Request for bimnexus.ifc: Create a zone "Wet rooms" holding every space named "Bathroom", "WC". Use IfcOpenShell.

First a look at what the model holds.

```python
import ifcopenshell

model = ifcopenshell.open("bimnexus.ifc")
print(model.schema)
seen = {}
for space in model.by_type("IfcSpace"):
    seen[space.LongName] = seen.get(space.LongName, 0) + 1
for name, count in sorted(seen.items(), key=str):
    print(count, "x", name)
print("zones:", [z.Name for z in model.by_type("IfcZone")][:20])
```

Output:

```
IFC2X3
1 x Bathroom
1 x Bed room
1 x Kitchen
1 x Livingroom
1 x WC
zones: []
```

```python
import ifcopenshell
import ifcopenshell.api.group
import ifcopenshell.api.root

model = ifcopenshell.open("bimnexus.ifc")

names = {"Bathroom", "WC"}
spaces = [s for s in model.by_type("IfcSpace") if s.LongName in names]

zone = ifcopenshell.api.root.create_entity(model, ifc_class="IfcZone", name="Wet rooms")
ifcopenshell.api.group.assign_group(model, products=spaces, group=zone)
print(len(spaces), "spaces in", zone.Name)

model.write("bimnexus_rev.ifc")
```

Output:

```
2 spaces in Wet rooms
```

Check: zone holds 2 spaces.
